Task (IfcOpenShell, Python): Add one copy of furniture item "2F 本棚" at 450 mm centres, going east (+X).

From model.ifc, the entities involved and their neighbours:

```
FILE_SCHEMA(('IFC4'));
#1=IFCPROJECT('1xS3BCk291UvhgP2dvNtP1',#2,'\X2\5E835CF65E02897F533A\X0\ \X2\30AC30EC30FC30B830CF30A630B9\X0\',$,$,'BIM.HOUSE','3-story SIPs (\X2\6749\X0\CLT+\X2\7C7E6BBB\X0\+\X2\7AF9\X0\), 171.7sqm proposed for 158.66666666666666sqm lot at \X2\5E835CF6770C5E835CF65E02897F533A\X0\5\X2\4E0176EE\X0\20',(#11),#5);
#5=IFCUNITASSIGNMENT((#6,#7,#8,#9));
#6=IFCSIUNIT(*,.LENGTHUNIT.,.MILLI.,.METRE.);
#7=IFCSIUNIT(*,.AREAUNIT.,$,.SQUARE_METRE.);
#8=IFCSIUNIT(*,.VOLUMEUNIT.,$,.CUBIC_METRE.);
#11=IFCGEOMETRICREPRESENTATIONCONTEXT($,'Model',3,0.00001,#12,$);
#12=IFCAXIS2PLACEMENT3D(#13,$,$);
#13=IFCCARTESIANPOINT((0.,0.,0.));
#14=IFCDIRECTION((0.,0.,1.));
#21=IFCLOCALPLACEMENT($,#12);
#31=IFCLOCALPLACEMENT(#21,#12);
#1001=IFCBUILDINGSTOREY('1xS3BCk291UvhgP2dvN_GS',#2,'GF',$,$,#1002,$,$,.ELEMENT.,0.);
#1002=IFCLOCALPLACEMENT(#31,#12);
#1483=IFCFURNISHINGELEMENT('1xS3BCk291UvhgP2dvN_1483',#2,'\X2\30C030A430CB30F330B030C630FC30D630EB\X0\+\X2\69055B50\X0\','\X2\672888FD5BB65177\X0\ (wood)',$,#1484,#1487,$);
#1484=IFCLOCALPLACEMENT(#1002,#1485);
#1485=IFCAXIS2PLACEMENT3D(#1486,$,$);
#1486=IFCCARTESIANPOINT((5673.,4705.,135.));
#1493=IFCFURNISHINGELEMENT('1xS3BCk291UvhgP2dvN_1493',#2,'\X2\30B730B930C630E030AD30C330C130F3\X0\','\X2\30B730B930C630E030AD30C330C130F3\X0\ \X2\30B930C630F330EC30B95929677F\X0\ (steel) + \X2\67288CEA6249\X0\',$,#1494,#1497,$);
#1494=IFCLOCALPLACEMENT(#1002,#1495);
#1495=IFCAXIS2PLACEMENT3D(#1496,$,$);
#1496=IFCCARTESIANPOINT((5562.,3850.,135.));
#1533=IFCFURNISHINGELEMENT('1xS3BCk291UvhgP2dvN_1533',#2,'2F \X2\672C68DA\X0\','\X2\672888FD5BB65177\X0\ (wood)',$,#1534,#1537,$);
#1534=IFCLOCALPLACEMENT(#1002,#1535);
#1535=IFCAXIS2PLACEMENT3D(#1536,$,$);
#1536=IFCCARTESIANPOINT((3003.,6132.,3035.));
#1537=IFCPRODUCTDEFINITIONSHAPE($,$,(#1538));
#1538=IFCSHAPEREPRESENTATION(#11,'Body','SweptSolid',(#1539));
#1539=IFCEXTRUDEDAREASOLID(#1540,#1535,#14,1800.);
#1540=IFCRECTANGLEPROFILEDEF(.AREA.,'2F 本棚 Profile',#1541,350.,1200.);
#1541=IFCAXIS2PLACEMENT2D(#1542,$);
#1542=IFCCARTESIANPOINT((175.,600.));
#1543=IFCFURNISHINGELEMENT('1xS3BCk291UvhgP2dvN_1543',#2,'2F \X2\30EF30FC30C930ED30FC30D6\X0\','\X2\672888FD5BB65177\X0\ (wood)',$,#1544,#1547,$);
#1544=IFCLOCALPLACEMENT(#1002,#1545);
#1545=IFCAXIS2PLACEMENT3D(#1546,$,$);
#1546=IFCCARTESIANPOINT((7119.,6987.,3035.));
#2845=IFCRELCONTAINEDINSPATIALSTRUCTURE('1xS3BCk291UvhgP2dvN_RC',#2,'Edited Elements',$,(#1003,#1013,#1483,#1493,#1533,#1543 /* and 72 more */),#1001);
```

```python
import numpy as np
import ifcopenshell
import ifcopenshell.api.geometry
import ifcopenshell.api.root
import ifcopenshell.util.element
import ifcopenshell.util.placement

model = ifcopenshell.open("model.ifc")


def reuse_history(source, copy):
    """copy_class also copies each property set's owner history, people and application; keep the originals."""
    for rel in copy.IsDefinedBy:
        if rel.is_a("IfcRelDefinesByProperties") and (history := rel.RelatingPropertyDefinition.OwnerHistory):
            rel.RelatingPropertyDefinition.OwnerHistory = source.OwnerHistory
            ifcopenshell.util.element.remove_deep2(model, history)


source = model.by_guid("1xS3BCk291UvhgP2dvN_1533")
base = ifcopenshell.util.placement.get_local_placement(source.ObjectPlacement)
step = np.array([1.0, 0.0, 0.0]) * 450.0

for i in range(1, 2):
    copy = ifcopenshell.api.root.copy_class(model, product=source)
    copy.Representation = ifcopenshell.util.element.copy_deep(
        model, source.Representation, exclude=["IfcGeometricRepresentationContext", "IfcRepresentationMap"]
    )
    reuse_history(source, copy)
    matrix = base.copy()
    matrix[:3, 3] += i * step
    print("added at", matrix[:3, 3].round(3) + 0.0)
    ifcopenshell.api.geometry.edit_object_placement(model, product=copy, matrix=matrix, is_si=False)

model.write("model_edited.ifc")
```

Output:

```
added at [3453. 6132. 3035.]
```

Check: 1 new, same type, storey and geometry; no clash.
